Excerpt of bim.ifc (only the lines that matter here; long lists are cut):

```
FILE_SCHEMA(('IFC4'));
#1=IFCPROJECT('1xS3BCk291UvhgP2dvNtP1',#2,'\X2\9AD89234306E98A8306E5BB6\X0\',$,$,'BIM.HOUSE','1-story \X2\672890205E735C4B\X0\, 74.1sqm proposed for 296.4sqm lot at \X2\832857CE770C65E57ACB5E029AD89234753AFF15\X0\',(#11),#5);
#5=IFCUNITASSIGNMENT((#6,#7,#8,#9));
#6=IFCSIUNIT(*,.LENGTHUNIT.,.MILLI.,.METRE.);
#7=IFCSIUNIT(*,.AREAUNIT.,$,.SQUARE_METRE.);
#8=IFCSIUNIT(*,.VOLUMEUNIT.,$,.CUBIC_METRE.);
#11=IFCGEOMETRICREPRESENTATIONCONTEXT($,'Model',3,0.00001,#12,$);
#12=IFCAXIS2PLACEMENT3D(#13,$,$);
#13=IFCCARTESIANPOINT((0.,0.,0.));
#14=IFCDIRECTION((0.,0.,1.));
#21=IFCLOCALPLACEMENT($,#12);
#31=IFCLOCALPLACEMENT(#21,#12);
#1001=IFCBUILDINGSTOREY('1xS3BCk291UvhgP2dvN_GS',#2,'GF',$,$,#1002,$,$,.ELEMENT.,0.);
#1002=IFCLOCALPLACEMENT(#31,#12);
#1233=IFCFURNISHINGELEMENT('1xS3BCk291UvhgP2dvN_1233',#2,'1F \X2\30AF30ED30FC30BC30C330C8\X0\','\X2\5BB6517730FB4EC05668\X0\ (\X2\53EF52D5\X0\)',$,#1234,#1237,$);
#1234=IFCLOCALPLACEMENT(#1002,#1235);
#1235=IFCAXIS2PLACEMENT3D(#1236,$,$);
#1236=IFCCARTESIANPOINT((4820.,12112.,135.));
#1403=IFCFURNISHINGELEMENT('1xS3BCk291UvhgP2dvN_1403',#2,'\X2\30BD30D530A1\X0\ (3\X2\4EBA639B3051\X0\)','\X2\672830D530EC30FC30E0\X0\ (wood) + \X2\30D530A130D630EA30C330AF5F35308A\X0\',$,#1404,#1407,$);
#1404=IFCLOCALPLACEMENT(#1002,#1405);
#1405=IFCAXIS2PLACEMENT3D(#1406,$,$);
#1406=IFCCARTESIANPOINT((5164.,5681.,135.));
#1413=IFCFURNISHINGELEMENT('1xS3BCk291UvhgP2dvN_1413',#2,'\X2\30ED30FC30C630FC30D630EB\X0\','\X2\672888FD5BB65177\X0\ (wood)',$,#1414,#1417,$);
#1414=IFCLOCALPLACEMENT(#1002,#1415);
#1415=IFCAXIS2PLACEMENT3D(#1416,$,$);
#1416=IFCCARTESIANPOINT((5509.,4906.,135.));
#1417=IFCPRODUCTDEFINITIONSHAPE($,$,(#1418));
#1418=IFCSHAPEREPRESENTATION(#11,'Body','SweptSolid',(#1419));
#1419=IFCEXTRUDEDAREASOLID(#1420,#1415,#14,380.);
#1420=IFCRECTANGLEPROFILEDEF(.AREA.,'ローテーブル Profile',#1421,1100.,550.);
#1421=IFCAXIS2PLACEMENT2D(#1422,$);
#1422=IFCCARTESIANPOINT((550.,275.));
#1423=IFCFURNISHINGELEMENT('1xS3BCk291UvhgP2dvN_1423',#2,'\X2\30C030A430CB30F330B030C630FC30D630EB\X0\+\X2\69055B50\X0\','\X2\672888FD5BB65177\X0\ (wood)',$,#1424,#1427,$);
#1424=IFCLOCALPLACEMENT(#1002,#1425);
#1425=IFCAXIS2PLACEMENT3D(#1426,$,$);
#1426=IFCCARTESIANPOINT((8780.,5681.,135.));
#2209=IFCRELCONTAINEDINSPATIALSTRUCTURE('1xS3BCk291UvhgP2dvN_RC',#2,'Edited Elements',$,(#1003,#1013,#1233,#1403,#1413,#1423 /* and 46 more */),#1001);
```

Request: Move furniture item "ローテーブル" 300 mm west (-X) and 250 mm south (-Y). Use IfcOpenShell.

```python
import ifcopenshell
import ifcopenshell.api.geometry
import ifcopenshell.util.placement
import ifcopenshell.util.unit

model = ifcopenshell.open("bim.ifc")
unit_scale = ifcopenshell.util.unit.calculate_unit_scale(model)

item = model.by_guid("1xS3BCk291UvhgP2dvN_1413")
matrix = ifcopenshell.util.placement.get_local_placement(item.ObjectPlacement)
matrix[0, 3] -= 0.3 / unit_scale
matrix[1, 3] -= 0.25 / unit_scale
ifcopenshell.api.geometry.edit_object_placement(model, product=item, matrix=matrix, is_si=False)

print(ifcopenshell.util.placement.get_local_placement(item.ObjectPlacement).round(3) + 0.0)

model.write("bim_rev.ifc")
```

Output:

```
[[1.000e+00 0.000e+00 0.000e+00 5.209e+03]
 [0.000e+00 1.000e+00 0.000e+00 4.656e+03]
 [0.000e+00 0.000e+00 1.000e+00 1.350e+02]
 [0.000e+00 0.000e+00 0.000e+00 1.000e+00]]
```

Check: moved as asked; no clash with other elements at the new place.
